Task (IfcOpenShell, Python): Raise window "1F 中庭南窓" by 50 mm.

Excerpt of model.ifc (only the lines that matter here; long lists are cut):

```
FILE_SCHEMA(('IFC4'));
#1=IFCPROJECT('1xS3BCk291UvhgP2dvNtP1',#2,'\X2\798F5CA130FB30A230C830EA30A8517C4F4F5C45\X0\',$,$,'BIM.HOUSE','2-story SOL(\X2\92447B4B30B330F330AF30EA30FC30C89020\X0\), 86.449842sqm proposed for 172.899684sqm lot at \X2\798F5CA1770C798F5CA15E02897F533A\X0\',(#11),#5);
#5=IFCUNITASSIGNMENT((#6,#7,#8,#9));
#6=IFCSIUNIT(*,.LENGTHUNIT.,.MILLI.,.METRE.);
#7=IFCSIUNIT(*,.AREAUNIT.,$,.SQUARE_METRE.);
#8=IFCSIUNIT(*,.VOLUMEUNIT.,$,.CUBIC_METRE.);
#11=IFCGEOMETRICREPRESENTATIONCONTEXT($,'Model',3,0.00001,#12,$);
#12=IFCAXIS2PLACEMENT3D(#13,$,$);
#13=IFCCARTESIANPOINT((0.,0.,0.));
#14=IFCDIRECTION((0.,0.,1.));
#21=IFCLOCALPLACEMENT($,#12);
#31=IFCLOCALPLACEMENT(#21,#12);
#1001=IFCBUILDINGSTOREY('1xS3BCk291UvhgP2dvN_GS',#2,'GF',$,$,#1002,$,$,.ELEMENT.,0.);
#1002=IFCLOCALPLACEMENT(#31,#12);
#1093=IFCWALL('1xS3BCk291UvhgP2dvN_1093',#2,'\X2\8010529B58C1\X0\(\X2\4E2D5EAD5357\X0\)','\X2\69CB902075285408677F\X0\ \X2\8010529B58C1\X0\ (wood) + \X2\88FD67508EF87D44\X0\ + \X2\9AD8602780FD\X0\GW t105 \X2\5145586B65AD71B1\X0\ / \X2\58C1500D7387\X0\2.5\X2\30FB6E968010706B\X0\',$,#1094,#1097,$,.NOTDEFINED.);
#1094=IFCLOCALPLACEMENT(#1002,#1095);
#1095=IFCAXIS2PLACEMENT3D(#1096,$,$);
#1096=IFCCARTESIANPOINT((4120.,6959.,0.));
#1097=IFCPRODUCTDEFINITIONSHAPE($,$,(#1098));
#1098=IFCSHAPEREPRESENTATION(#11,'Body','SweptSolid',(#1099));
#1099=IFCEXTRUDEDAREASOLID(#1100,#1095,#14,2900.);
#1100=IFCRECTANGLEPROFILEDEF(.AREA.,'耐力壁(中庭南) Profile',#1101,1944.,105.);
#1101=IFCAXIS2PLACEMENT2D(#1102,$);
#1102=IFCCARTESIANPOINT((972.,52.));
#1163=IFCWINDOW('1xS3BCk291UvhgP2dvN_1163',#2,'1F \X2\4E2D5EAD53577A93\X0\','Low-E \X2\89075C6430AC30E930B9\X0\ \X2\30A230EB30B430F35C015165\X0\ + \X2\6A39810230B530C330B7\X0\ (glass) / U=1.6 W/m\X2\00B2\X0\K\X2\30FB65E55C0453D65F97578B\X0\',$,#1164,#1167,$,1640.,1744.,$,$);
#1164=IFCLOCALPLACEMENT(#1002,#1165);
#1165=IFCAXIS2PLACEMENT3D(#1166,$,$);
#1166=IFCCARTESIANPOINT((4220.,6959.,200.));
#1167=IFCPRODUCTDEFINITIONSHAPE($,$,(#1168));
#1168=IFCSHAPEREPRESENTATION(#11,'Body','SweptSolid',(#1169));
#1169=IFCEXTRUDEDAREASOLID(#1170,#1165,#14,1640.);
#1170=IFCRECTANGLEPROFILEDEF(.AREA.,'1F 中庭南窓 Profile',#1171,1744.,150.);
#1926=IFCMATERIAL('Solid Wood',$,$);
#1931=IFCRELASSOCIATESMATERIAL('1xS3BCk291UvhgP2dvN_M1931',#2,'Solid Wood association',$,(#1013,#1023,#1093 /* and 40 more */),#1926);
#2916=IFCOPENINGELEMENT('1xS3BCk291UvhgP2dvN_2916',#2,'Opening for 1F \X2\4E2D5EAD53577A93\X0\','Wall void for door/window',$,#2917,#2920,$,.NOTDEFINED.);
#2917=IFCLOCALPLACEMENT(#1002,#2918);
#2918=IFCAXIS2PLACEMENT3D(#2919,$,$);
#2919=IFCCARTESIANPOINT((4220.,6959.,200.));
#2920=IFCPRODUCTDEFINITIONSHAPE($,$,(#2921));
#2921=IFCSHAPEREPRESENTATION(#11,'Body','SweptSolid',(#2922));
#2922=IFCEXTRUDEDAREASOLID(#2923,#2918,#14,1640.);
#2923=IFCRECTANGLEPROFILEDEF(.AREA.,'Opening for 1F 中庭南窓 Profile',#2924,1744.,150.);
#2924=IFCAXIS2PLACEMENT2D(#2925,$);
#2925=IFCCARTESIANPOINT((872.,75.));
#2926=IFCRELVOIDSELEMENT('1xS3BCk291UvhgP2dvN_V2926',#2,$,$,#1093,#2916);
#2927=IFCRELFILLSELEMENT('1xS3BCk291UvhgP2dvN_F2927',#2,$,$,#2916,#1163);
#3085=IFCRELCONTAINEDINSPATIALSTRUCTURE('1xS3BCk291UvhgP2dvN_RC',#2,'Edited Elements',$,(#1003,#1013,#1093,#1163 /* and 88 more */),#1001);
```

```python
import numpy as np
import ifcopenshell
import ifcopenshell.api.geometry
import ifcopenshell.util.placement
import ifcopenshell.util.unit

model = ifcopenshell.open("model.ifc")
unit_scale = ifcopenshell.util.unit.calculate_unit_scale(model)

window = model.by_id(1163)
opening = window.FillsVoids[0].RelatingOpeningElement
dz = 50.0

shift = np.array([0.0, 0.0, dz])
# The window is not placed relative to its opening, so move both.
for product in (opening, window):
    matrix = ifcopenshell.util.placement.get_local_placement(product.ObjectPlacement)
    matrix[:3, 3] += shift
    ifcopenshell.api.geometry.edit_object_placement(model, product=product, matrix=matrix, is_si=False)

print(f"moved by {dz * unit_scale:+.3f} m")

model.write("model_rev.ifc")
```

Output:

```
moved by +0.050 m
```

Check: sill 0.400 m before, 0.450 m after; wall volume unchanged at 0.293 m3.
